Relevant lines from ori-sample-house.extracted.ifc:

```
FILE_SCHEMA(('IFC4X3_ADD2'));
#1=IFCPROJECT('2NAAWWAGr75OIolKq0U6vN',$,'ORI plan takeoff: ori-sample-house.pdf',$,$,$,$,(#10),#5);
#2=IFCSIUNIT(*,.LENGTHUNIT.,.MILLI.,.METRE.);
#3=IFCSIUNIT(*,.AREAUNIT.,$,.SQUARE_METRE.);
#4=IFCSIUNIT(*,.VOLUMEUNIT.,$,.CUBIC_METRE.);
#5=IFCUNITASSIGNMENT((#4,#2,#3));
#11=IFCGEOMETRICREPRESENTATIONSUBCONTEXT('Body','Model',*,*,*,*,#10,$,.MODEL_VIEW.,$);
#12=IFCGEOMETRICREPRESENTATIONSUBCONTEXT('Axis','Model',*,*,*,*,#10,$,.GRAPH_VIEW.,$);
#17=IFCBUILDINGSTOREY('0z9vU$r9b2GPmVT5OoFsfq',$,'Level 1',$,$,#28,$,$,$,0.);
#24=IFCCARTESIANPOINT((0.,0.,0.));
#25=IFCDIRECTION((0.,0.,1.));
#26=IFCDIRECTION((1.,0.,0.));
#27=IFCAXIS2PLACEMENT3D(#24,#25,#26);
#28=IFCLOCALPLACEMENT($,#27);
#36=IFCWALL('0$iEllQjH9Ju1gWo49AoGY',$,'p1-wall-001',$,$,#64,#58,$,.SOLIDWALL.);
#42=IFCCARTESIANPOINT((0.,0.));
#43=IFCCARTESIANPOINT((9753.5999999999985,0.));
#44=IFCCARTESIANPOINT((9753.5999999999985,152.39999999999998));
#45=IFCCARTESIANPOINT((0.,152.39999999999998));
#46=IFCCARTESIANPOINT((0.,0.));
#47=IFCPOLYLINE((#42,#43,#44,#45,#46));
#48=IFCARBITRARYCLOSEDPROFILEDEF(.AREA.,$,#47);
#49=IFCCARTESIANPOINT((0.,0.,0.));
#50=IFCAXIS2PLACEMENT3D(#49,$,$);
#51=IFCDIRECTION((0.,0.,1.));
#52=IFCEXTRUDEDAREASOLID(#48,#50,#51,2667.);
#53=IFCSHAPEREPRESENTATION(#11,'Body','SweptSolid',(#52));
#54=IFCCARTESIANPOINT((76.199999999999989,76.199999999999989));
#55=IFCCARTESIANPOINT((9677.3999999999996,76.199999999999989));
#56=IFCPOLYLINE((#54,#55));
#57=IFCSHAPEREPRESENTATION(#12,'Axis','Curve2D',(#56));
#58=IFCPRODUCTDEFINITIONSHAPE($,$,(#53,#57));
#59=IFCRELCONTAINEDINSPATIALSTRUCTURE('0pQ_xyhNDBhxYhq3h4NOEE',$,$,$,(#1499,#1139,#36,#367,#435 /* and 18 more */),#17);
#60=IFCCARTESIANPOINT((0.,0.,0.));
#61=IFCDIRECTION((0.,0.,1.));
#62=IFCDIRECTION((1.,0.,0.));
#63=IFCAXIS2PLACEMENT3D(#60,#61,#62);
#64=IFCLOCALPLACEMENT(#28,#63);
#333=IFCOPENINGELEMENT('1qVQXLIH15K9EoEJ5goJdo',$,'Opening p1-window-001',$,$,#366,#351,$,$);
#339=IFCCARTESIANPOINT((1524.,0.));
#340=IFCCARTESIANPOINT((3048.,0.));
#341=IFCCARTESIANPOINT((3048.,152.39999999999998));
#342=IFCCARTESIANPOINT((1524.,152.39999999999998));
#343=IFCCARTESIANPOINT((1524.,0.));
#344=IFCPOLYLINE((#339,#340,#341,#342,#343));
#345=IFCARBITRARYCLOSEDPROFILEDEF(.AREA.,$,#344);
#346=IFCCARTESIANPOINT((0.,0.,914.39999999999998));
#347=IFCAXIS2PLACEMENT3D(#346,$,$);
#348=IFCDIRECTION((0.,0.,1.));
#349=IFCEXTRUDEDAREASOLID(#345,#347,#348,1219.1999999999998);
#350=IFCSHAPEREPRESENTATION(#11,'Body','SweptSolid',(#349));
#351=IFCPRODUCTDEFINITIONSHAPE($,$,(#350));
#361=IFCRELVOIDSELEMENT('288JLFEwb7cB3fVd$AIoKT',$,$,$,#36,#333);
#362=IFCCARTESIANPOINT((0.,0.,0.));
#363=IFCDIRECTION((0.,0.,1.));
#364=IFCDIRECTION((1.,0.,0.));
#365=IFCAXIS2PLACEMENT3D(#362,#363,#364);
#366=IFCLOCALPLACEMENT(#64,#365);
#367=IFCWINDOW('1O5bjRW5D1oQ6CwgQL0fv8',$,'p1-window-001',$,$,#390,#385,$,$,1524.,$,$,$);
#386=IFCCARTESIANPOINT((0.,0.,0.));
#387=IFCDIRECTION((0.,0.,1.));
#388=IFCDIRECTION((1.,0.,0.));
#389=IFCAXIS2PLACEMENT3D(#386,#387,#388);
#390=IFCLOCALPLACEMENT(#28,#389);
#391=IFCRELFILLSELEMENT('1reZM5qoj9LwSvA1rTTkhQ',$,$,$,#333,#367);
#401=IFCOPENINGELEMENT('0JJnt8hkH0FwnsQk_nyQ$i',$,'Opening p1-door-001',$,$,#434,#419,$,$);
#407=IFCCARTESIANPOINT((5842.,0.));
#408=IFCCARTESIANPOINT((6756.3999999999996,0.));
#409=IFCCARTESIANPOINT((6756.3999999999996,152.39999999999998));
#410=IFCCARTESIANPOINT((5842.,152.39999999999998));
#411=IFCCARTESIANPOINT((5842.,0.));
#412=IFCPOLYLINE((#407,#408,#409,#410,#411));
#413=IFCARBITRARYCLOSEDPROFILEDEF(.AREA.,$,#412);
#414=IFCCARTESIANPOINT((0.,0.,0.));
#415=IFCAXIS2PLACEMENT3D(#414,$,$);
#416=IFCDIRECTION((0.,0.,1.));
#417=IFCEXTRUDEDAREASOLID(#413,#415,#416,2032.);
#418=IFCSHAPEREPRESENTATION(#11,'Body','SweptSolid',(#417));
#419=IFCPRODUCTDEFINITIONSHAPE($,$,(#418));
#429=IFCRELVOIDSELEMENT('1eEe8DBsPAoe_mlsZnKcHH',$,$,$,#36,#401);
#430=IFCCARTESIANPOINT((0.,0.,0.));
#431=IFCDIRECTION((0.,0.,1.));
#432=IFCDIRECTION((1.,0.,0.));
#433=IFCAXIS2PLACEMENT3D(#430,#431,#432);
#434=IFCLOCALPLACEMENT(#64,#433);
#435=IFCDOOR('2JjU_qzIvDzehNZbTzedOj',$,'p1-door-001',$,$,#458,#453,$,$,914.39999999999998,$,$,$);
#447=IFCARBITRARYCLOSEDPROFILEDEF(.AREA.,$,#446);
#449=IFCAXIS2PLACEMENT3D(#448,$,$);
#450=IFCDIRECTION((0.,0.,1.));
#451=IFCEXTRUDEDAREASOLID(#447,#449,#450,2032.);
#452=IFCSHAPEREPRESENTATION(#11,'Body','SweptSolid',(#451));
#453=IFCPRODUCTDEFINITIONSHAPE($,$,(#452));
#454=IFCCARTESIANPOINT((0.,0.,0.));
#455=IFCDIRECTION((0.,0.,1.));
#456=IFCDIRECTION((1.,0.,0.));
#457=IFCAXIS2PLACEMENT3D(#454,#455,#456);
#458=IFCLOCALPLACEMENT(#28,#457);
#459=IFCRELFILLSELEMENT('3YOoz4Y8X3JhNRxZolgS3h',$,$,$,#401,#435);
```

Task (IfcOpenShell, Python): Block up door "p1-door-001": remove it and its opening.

```python
import ifcopenshell
import ifcopenshell.api.feature
import ifcopenshell.api.root
import ifcopenshell.geom
import ifcopenshell.util.shape

model = ifcopenshell.open("ori-sample-house.extracted.ifc")
settings = ifcopenshell.geom.settings()


def volume(element):
    """Net volume in cubic metres, openings subtracted."""
    shape = ifcopenshell.geom.create_shape(settings, element)
    return ifcopenshell.util.shape.get_volume(shape.geometry)


door = model.by_id(435)
opening = door.FillsVoids[0].RelatingOpeningElement
wall = opening.VoidsElements[0].RelatingBuildingElement
before = volume(wall)

ifcopenshell.api.root.remove_product(model, product=door)
ifcopenshell.api.feature.remove_feature(model, feature=opening)

after = volume(wall)

print(f"wall volume {before:.3f} -> {after:.3f} m3")

model.write("ori-sample-house.extracted_edited.ifc")
```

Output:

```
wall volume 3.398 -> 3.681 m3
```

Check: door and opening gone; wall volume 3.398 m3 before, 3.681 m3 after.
